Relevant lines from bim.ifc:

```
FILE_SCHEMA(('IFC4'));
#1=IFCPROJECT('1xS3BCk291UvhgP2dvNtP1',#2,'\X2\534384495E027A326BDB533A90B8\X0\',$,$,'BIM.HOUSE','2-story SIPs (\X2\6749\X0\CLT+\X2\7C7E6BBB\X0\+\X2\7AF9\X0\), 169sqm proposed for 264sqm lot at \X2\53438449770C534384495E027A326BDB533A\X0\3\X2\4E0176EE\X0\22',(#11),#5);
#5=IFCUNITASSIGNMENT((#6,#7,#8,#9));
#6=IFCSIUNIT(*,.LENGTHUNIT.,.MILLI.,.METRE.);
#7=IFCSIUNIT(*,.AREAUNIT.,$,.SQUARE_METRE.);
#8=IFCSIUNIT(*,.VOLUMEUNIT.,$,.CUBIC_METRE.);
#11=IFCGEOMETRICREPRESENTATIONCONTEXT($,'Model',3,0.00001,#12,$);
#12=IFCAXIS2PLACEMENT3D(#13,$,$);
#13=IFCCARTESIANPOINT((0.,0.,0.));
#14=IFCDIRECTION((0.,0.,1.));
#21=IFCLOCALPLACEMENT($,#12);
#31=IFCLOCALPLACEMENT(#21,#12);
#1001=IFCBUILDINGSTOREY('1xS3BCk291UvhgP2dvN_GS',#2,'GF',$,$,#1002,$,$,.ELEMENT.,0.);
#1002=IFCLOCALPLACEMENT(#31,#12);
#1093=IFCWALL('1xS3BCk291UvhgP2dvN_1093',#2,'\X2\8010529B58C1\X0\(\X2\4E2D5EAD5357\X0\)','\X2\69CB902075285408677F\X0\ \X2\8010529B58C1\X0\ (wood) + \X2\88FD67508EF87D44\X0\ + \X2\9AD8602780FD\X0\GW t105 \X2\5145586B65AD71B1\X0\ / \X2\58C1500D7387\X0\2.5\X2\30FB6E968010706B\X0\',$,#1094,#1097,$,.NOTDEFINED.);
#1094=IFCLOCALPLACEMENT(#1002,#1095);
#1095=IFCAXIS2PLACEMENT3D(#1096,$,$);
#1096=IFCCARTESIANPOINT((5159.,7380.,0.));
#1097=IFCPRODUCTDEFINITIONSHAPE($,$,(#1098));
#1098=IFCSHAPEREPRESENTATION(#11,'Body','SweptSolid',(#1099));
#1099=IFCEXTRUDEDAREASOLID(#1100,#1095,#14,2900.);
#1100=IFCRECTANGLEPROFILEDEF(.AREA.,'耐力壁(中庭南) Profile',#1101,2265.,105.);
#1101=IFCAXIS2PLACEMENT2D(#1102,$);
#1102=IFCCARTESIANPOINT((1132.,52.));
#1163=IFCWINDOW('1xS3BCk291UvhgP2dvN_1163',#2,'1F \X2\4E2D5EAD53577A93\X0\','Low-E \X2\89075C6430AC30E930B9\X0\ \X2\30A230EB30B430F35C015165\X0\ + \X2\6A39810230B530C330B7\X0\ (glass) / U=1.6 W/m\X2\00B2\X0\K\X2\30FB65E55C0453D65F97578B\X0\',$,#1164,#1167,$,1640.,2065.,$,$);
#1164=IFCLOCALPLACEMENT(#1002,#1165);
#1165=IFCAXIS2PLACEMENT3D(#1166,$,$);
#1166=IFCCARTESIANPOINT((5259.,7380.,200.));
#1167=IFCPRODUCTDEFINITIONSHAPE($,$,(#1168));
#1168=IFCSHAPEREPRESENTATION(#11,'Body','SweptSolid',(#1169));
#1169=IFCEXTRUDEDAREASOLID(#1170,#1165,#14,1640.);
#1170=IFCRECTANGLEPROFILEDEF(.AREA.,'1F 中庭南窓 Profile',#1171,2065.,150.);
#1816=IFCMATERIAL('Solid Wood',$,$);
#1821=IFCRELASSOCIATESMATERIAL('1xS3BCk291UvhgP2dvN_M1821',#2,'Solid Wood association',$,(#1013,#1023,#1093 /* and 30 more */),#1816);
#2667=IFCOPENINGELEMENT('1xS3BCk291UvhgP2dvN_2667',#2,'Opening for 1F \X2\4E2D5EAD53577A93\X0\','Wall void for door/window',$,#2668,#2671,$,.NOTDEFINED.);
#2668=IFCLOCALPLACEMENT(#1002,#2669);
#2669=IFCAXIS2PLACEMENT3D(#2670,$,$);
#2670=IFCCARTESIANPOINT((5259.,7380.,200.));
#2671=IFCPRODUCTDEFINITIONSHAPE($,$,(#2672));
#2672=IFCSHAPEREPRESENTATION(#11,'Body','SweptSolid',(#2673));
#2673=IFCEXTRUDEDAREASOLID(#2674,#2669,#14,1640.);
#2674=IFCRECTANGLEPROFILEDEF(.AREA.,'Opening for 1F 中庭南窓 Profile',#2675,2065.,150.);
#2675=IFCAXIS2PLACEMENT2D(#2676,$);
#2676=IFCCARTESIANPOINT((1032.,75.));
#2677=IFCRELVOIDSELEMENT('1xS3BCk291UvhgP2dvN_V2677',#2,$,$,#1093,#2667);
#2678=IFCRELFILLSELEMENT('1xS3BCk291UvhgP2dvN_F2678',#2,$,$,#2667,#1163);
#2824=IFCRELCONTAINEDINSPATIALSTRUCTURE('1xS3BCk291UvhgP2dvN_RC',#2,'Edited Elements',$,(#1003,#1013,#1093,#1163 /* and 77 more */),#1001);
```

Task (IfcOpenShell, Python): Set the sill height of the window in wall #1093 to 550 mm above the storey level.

```python
import numpy as np
import ifcopenshell
import ifcopenshell.api.geometry
import ifcopenshell.geom
import ifcopenshell.util.element
import ifcopenshell.util.placement
import ifcopenshell.util.shape
import ifcopenshell.util.unit

model = ifcopenshell.open("bim.ifc")
unit_scale = ifcopenshell.util.unit.calculate_unit_scale(model)

window = model.by_guid("1xS3BCk291UvhgP2dvN_1163")
opening = window.FillsVoids[0].RelatingOpeningElement
storey = ifcopenshell.util.element.get_container(window, ifc_class="IfcBuildingStorey")
level = ifcopenshell.util.placement.get_local_placement(storey.ObjectPlacement)[2, 3]

# The opening's origin need not be at the sill, so measure its lowest point.
shape = ifcopenshell.geom.create_shape(ifcopenshell.geom.settings(), opening)
bottom = ifcopenshell.util.shape.get_shape_bottom_elevation(shape, shape.geometry) / unit_scale
dz = level + 550.0 - bottom

shift = np.array([0.0, 0.0, dz])
# The window is not placed relative to its opening, so move both.
for product in (opening, window):
    matrix = ifcopenshell.util.placement.get_local_placement(product.ObjectPlacement)
    matrix[:3, 3] += shift
    ifcopenshell.api.geometry.edit_object_placement(model, product=product, matrix=matrix, is_si=False)

print(f"moved by {dz * unit_scale:+.3f} m")

model.write("bim_v2.ifc")
```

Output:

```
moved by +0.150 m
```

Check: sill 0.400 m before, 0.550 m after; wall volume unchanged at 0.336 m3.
